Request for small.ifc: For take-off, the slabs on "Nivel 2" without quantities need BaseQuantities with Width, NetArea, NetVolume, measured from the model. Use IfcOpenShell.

First a look at what the model holds.

```python
import ifcopenshell
import ifcopenshell.util.element
import ifcopenshell.util.unit

model = ifcopenshell.open("small.ifc")
print(model.schema)
for unit_type in ("LENGTHUNIT", "AREAUNIT", "VOLUMEUNIT"):
    print(unit_type, ifcopenshell.util.unit.calculate_unit_scale(model, unit_type))
storey = next(s for s in model.by_type("IfcBuildingStorey") if s.Name == "Nivel 2")
slabs = [e for e in ifcopenshell.util.element.get_decomposition(storey) if e.is_a("IfcSlab")]
for e in sorted(slabs, key=lambda e: e.id()):
    print(e.id(), e.is_a(), e.Name, list(ifcopenshell.util.element.get_psets(e, qtos_only=True)), sep=" | ")
```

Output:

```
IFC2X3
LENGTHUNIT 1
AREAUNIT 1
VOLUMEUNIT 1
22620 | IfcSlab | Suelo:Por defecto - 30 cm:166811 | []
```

```python
import ifcopenshell
import ifcopenshell.api.pset
import ifcopenshell.geom
import ifcopenshell.util.element
import ifcopenshell.util.shape
import ifcopenshell.util.unit

model = ifcopenshell.open("small.ifc")
unit_scale = ifcopenshell.util.unit.calculate_unit_scale(model)
area_scale = ifcopenshell.util.unit.calculate_unit_scale(model, "AREAUNIT")
volume_scale = ifcopenshell.util.unit.calculate_unit_scale(model, "VOLUMEUNIT")
settings = ifcopenshell.geom.settings()

storey = next(s for s in model.by_type("IfcBuildingStorey") if s.Name == "Nivel 2")
slabs = [e for e in ifcopenshell.util.element.get_decomposition(storey) if e.is_a("IfcSlab")]

for e in sorted(slabs, key=lambda e: e.id()):
    if ifcopenshell.util.element.get_psets(e, qtos_only=True, should_inherit=False):
        continue
    # Geometry comes back in metres, in the element's own axes.
    shape = ifcopenshell.geom.create_shape(settings, e)
    values = {
        "Width": ifcopenshell.util.shape.get_z(shape.geometry) / unit_scale,
        "NetArea": ifcopenshell.util.shape.get_footprint_area(shape.geometry) / area_scale,
        "NetVolume": ifcopenshell.util.shape.get_volume(shape.geometry) / volume_scale,
    }
    qto = ifcopenshell.api.pset.add_qto(model, product=e, name="BaseQuantities")
    ifcopenshell.api.pset.edit_qto(model, qto=qto, properties=values)
    print(e.id(), {k: round(v, 3) for k, v in values.items()})

model.write("small_rev.ifc")
```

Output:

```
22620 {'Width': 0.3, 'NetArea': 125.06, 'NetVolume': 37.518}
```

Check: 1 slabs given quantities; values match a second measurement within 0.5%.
